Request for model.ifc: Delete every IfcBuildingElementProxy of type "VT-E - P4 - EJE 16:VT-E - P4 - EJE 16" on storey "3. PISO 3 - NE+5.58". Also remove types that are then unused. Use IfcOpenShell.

First a look at what the model holds.

```python
import ifcopenshell
import ifcopenshell.util.element

model = ifcopenshell.open("model.ifc")
print(model.schema)
storey = next(s for s in model.by_type("IfcBuildingStorey") if s.Name == "3. PISO 3 - NE+5.58")
proxies = [e for e in ifcopenshell.util.element.get_decomposition(storey) if e.is_a("IfcBuildingElementProxy")]
seen = {}
for e in proxies:
    element_type = ifcopenshell.util.element.get_type(e)
    name = element_type.Name if element_type not in (None, e) else None
    seen[name] = seen.get(name, 0) + 1
for name, count in sorted(seen.items(), key=str):
    print(count, "x", name)
```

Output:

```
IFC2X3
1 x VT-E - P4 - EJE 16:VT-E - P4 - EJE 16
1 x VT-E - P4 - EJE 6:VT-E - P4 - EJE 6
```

```python
import ifcopenshell
import ifcopenshell.api.root
import ifcopenshell.util.element

model = ifcopenshell.open("model.ifc")

storey = next(s for s in model.by_type("IfcBuildingStorey") if s.Name == "3. PISO 3 - NE+5.58")
proxies = [e for e in ifcopenshell.util.element.get_decomposition(storey) if e.is_a("IfcBuildingElementProxy")]
targets = [e for e in proxies if (t := ifcopenshell.util.element.get_type(e)) not in (None, e) and t.Name == "VT-E - P4 - EJE 16:VT-E - P4 - EJE 16"]
types = {ifcopenshell.util.element.get_type(e) for e in targets} - {None, *targets}

for e in targets:
    ifcopenshell.api.root.remove_product(model, product=e)
print(len(targets), "removed")

unused = [t for t in types if not ifcopenshell.util.element.get_types(t)]
for t in unused:
    ifcopenshell.api.root.remove_product(model, product=t)
print(len(unused), "unused types removed")

model.write("model_edited.ifc")
```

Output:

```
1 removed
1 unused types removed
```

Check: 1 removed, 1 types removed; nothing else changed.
